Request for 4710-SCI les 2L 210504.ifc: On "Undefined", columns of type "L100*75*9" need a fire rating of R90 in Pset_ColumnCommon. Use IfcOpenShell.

First a look at what the model holds.

```python
import ifcopenshell
import ifcopenshell.util.element

model = ifcopenshell.open("4710-SCI les 2L 210504.ifc")
print(model.schema)
storey = next(s for s in model.by_type("IfcBuildingStorey") if s.Name == "Undefined")
columns = [e for e in ifcopenshell.util.element.get_decomposition(storey) if e.is_a("IfcColumn")]
seen = {}
for e in columns:
    element_type = ifcopenshell.util.element.get_type(e)
    key = (element_type.Name if element_type != e and element_type else None, ifcopenshell.util.element.get_pset(e, "Pset_ColumnCommon", "FireRating"))
    seen[key] = seen.get(key, 0) + 1
for (name, value), count in sorted(seen.items(), key=str):
    print(count, "x", name, "|", value)
```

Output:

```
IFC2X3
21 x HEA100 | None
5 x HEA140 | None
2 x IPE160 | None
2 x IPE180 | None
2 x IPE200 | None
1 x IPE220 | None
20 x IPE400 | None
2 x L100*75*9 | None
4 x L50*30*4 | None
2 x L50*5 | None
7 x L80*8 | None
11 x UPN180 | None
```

```python
import ifcopenshell
import ifcopenshell.api.pset
import ifcopenshell.util.element

model = ifcopenshell.open("4710-SCI les 2L 210504.ifc")

storey = next(s for s in model.by_type("IfcBuildingStorey") if s.Name == "Undefined")
columns = [e for e in ifcopenshell.util.element.get_decomposition(storey) if e.is_a("IfcColumn")]

count = 0
for e in columns:
    element_type = ifcopenshell.util.element.get_type(e)
    if element_type in (None, e) or element_type.Name != "L100*75*9":
        continue
    found = ifcopenshell.util.element.get_pset(e, "Pset_ColumnCommon", should_inherit=False)
    if found:
        pset = model.by_id(found["id"])
        if len(ifcopenshell.util.element.get_elements_by_pset(pset)) > 1:
            pset = ifcopenshell.api.pset.unshare_pset(model, products=[e], pset=pset)[0]
    else:
        pset = ifcopenshell.api.pset.add_pset(model, product=e, name="Pset_ColumnCommon")
    ifcopenshell.api.pset.edit_pset(model, pset=pset, properties={"FireRating": "R90"})
    count += 1

print(count, "columns updated")

model.write("4710-SCI les 2L 210504_v2.ifc")
```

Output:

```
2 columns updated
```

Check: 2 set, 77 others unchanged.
